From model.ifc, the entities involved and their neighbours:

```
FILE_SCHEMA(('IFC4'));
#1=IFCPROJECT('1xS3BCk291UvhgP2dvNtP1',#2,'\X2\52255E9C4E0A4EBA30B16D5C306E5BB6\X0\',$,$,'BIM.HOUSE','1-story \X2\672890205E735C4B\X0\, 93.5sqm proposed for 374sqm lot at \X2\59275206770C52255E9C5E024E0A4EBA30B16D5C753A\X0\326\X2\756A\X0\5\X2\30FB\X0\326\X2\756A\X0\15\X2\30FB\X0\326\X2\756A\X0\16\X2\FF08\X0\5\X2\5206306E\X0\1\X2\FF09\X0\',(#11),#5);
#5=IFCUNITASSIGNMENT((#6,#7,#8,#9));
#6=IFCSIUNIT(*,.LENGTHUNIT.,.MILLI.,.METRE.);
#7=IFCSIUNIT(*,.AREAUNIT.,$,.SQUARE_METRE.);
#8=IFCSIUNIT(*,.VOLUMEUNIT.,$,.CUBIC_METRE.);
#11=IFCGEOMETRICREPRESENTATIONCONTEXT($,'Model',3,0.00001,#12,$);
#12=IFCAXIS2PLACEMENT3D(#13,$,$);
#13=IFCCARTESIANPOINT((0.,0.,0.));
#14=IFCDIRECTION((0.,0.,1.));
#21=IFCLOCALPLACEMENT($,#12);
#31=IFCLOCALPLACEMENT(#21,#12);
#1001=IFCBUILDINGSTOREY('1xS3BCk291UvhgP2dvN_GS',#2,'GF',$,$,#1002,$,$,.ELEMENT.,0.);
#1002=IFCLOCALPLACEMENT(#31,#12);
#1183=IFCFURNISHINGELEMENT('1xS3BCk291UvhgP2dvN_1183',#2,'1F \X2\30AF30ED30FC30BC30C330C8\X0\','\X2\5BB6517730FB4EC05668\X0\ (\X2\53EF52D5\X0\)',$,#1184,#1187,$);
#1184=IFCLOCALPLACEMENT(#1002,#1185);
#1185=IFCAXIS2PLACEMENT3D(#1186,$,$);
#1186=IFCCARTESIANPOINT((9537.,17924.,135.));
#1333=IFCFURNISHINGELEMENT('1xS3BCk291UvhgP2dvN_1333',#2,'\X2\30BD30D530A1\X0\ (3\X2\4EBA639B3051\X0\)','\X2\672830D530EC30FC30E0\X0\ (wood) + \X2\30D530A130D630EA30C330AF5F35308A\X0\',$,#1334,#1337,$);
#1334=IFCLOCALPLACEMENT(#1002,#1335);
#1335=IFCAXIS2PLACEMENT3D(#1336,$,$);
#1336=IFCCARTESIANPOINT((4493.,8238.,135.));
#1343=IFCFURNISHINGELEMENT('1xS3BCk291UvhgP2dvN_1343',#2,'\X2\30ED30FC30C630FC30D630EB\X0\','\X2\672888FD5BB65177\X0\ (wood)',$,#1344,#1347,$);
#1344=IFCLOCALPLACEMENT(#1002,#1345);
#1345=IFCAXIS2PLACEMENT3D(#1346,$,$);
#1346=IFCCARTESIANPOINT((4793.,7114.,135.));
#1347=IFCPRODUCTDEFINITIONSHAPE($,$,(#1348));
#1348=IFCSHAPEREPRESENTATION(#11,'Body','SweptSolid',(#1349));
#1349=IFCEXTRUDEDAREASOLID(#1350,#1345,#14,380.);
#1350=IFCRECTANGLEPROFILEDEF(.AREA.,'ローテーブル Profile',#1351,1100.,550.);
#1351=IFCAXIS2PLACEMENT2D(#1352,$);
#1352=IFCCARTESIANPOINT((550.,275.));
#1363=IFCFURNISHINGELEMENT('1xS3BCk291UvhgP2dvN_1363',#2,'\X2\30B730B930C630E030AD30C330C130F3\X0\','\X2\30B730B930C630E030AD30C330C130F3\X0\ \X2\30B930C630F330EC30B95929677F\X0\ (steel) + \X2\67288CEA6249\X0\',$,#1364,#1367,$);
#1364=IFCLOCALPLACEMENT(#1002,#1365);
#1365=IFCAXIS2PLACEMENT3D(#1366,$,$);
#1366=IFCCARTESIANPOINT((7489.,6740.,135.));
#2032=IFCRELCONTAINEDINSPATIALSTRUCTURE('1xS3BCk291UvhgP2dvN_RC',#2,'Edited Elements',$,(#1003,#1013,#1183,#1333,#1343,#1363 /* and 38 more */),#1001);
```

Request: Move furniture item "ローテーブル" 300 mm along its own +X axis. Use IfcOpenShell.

```python
import ifcopenshell
import ifcopenshell.api.geometry
import ifcopenshell.util.placement
import ifcopenshell.util.unit

model = ifcopenshell.open("model.ifc")
unit_scale = ifcopenshell.util.unit.calculate_unit_scale(model)

item = model.by_guid("1xS3BCk291UvhgP2dvN_1343")
matrix = ifcopenshell.util.placement.get_local_placement(item.ObjectPlacement)
matrix[:3, 3] += matrix[:3, 0] * 0.3 / unit_scale
ifcopenshell.api.geometry.edit_object_placement(model, product=item, matrix=matrix, is_si=False)

print(ifcopenshell.util.placement.get_local_placement(item.ObjectPlacement).round(3) + 0.0)

model.write("model_edited.ifc")
```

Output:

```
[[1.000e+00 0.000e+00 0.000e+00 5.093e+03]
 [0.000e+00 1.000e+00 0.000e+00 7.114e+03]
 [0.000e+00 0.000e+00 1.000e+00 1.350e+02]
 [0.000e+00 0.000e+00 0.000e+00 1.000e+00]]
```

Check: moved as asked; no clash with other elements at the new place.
